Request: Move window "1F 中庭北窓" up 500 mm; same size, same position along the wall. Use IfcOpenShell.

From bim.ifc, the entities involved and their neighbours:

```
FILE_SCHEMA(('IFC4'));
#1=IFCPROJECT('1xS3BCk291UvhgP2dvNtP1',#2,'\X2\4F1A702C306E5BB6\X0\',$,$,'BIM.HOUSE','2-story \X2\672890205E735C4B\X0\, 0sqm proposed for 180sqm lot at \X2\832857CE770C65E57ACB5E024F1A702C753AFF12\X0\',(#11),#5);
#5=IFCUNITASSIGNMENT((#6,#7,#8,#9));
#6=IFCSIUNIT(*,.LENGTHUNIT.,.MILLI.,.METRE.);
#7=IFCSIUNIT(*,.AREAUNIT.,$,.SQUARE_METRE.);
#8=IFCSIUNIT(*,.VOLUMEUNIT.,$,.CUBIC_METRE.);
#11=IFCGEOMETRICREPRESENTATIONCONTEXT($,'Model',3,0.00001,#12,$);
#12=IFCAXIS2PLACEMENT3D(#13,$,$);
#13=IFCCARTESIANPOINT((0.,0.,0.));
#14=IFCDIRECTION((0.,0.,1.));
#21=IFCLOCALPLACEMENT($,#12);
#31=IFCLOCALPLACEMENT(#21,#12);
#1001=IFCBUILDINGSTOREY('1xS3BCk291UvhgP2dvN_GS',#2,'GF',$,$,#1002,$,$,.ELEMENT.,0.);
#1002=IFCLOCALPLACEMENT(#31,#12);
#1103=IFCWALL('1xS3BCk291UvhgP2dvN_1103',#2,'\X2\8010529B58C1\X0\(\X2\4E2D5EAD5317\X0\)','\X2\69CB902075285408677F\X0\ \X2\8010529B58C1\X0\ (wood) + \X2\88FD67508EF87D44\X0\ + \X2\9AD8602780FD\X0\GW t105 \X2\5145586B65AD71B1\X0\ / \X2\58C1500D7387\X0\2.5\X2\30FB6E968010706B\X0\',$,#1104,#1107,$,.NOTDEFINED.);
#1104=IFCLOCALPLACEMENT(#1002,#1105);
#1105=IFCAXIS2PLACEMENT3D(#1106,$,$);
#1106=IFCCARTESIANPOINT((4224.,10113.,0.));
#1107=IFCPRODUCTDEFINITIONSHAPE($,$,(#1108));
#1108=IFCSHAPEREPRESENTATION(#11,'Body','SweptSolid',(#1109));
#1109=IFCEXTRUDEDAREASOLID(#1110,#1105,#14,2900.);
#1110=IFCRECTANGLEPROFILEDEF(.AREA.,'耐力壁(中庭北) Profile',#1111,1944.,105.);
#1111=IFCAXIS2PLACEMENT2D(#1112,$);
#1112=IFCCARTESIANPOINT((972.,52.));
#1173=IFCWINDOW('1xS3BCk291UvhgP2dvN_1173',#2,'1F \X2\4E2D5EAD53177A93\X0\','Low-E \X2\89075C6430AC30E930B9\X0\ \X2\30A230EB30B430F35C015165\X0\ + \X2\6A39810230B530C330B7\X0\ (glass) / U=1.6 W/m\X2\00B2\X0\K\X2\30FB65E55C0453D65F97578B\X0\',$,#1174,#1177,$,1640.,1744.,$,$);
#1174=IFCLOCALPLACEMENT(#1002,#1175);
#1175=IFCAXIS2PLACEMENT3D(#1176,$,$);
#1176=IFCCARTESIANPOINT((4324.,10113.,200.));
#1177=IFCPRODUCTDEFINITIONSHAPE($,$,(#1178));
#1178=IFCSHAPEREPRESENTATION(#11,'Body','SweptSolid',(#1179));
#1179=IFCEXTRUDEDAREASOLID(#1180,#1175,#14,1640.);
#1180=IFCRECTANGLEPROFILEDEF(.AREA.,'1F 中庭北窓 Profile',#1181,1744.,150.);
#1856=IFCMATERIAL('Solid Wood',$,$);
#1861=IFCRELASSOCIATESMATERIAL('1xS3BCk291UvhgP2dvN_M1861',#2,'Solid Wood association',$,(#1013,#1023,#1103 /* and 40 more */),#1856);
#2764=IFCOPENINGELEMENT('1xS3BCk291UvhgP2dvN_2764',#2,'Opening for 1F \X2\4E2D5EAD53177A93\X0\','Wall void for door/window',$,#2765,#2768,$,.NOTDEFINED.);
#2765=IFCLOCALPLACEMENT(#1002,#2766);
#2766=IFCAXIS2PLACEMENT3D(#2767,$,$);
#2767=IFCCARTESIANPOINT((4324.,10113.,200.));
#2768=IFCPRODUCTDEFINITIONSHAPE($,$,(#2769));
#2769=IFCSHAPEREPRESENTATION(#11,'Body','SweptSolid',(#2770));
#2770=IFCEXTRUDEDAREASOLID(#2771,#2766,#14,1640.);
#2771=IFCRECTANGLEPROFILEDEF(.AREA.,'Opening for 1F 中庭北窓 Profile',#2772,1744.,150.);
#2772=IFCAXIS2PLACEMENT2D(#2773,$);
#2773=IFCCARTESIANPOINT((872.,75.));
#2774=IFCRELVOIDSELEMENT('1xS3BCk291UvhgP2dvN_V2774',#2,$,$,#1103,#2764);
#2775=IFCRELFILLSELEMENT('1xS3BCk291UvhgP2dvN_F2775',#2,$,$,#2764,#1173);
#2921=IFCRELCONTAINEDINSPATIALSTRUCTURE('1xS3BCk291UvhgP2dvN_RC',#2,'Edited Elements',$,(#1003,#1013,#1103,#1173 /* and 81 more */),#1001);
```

```python
import numpy as np
import ifcopenshell
import ifcopenshell.api.geometry
import ifcopenshell.util.placement
import ifcopenshell.util.unit

model = ifcopenshell.open("bim.ifc")
unit_scale = ifcopenshell.util.unit.calculate_unit_scale(model)

window = model.by_guid("1xS3BCk291UvhgP2dvN_1173")
opening = window.FillsVoids[0].RelatingOpeningElement
dz = 0.5 / unit_scale

shift = np.array([0.0, 0.0, dz])
# The window is not placed relative to its opening, so move both.
for product in (opening, window):
    matrix = ifcopenshell.util.placement.get_local_placement(product.ObjectPlacement)
    matrix[:3, 3] += shift
    ifcopenshell.api.geometry.edit_object_placement(model, product=product, matrix=matrix, is_si=False)

print(f"moved by {dz * unit_scale:+.3f} m")

model.write("bim-out.ifc")
```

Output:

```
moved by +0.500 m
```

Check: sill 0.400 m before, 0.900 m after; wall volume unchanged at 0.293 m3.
